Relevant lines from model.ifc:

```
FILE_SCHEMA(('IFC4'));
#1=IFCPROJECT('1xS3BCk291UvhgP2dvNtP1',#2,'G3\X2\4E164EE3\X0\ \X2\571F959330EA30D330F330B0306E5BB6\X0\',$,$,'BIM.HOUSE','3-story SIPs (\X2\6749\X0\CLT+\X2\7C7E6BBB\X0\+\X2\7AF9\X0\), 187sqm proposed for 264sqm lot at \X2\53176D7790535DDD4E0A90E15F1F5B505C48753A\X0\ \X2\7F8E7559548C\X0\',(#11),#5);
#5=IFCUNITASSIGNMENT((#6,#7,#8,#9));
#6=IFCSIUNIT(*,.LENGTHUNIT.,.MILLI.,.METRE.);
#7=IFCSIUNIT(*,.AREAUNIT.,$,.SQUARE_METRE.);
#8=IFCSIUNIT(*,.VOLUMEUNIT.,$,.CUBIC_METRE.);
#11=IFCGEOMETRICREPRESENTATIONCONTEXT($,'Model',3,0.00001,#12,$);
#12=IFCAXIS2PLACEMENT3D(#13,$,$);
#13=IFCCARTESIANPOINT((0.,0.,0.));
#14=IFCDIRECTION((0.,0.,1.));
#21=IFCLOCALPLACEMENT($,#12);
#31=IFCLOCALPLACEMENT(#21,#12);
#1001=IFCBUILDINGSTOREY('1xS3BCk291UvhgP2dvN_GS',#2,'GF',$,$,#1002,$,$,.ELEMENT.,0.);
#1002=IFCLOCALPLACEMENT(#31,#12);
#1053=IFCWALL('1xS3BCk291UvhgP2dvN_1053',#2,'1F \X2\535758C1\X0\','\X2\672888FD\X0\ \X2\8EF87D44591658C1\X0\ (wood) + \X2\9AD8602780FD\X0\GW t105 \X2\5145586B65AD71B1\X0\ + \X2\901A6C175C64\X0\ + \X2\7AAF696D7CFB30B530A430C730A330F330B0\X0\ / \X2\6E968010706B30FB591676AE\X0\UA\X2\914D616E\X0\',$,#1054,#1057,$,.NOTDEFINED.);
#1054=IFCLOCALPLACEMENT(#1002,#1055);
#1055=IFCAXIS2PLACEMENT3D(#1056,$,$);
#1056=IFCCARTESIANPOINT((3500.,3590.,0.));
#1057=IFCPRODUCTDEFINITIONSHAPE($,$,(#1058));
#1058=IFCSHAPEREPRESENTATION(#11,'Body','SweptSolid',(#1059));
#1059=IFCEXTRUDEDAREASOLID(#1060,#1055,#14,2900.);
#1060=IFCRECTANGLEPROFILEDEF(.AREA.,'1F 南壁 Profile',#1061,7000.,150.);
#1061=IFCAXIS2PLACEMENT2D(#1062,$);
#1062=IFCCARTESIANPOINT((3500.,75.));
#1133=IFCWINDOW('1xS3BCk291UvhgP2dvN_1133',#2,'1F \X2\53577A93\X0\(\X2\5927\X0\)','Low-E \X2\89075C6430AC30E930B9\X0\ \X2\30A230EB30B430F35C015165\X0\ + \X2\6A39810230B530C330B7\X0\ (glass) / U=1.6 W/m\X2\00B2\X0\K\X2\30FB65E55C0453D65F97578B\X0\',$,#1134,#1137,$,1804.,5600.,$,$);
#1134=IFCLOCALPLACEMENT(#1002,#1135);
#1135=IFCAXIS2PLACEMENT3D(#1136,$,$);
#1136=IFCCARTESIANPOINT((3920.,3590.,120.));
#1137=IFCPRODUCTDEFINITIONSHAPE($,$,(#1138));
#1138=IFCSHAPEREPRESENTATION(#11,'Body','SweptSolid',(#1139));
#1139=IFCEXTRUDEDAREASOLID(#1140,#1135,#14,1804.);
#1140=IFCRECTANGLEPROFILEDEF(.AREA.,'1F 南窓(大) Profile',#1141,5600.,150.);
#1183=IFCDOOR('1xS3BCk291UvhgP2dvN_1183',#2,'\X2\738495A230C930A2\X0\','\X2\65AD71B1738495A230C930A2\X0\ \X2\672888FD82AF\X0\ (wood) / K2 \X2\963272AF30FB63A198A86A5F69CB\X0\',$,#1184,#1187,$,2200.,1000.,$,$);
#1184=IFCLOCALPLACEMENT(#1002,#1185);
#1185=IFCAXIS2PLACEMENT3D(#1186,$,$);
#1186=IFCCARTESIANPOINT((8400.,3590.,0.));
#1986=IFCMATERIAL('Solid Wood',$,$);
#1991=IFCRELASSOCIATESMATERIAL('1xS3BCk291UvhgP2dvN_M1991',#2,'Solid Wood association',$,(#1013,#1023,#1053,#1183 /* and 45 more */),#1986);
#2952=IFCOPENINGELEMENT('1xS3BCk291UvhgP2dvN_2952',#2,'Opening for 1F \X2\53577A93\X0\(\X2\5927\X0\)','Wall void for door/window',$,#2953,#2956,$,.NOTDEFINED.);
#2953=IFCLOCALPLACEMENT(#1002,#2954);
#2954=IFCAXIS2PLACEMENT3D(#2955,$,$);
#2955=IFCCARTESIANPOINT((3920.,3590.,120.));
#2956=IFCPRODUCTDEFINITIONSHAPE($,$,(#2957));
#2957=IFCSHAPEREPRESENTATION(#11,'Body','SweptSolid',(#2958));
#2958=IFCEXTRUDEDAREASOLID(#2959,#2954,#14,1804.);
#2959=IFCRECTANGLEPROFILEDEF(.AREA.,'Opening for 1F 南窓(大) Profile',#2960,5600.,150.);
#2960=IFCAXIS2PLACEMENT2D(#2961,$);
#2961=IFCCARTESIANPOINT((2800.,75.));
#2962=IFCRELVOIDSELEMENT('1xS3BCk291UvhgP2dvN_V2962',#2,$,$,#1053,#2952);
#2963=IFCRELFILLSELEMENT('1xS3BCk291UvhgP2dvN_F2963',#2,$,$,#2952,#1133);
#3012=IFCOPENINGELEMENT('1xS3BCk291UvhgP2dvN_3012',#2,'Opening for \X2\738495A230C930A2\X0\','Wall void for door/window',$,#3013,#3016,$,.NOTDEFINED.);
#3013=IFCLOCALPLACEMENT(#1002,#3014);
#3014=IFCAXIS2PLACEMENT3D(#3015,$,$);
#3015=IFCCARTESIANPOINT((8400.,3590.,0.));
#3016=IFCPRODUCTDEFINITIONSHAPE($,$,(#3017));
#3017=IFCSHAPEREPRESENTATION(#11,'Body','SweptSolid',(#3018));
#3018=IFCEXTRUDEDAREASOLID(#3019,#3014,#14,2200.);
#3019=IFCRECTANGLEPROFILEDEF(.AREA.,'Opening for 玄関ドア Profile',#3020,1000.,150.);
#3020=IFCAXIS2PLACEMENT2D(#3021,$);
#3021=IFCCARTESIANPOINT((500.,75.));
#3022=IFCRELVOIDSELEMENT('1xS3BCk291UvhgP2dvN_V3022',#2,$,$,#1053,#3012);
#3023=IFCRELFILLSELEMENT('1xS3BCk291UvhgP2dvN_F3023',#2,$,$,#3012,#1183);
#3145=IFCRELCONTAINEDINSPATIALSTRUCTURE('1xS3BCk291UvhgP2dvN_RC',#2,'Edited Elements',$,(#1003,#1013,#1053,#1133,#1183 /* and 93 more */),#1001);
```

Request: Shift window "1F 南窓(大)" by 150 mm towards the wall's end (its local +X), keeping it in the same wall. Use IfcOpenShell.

```python
import ifcopenshell
import ifcopenshell.api.geometry
import ifcopenshell.util.placement

model = ifcopenshell.open("model.ifc")

window = model.by_guid("1xS3BCk291UvhgP2dvN_1133")
opening = window.FillsVoids[0].RelatingOpeningElement
wall = opening.VoidsElements[0].RelatingBuildingElement

wall_matrix = ifcopenshell.util.placement.get_local_placement(wall.ObjectPlacement)
shift = wall_matrix[:3, 0] * 150.0
before = ifcopenshell.util.placement.get_local_placement(window.ObjectPlacement)[:3, 3].copy()

# The window is not placed relative to its opening, so move both.
for product in (opening, window):
    matrix = ifcopenshell.util.placement.get_local_placement(product.ObjectPlacement)
    matrix[:3, 3] += shift
    ifcopenshell.api.geometry.edit_object_placement(model, product=product, matrix=matrix, is_si=False)

after = ifcopenshell.util.placement.get_local_placement(window.ObjectPlacement)[:3, 3]
print("window moved by", (after - before).round(3) + 0.0)

model.write("model_v2.ifc")
```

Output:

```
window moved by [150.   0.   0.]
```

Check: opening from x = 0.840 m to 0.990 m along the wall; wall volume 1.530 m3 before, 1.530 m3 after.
